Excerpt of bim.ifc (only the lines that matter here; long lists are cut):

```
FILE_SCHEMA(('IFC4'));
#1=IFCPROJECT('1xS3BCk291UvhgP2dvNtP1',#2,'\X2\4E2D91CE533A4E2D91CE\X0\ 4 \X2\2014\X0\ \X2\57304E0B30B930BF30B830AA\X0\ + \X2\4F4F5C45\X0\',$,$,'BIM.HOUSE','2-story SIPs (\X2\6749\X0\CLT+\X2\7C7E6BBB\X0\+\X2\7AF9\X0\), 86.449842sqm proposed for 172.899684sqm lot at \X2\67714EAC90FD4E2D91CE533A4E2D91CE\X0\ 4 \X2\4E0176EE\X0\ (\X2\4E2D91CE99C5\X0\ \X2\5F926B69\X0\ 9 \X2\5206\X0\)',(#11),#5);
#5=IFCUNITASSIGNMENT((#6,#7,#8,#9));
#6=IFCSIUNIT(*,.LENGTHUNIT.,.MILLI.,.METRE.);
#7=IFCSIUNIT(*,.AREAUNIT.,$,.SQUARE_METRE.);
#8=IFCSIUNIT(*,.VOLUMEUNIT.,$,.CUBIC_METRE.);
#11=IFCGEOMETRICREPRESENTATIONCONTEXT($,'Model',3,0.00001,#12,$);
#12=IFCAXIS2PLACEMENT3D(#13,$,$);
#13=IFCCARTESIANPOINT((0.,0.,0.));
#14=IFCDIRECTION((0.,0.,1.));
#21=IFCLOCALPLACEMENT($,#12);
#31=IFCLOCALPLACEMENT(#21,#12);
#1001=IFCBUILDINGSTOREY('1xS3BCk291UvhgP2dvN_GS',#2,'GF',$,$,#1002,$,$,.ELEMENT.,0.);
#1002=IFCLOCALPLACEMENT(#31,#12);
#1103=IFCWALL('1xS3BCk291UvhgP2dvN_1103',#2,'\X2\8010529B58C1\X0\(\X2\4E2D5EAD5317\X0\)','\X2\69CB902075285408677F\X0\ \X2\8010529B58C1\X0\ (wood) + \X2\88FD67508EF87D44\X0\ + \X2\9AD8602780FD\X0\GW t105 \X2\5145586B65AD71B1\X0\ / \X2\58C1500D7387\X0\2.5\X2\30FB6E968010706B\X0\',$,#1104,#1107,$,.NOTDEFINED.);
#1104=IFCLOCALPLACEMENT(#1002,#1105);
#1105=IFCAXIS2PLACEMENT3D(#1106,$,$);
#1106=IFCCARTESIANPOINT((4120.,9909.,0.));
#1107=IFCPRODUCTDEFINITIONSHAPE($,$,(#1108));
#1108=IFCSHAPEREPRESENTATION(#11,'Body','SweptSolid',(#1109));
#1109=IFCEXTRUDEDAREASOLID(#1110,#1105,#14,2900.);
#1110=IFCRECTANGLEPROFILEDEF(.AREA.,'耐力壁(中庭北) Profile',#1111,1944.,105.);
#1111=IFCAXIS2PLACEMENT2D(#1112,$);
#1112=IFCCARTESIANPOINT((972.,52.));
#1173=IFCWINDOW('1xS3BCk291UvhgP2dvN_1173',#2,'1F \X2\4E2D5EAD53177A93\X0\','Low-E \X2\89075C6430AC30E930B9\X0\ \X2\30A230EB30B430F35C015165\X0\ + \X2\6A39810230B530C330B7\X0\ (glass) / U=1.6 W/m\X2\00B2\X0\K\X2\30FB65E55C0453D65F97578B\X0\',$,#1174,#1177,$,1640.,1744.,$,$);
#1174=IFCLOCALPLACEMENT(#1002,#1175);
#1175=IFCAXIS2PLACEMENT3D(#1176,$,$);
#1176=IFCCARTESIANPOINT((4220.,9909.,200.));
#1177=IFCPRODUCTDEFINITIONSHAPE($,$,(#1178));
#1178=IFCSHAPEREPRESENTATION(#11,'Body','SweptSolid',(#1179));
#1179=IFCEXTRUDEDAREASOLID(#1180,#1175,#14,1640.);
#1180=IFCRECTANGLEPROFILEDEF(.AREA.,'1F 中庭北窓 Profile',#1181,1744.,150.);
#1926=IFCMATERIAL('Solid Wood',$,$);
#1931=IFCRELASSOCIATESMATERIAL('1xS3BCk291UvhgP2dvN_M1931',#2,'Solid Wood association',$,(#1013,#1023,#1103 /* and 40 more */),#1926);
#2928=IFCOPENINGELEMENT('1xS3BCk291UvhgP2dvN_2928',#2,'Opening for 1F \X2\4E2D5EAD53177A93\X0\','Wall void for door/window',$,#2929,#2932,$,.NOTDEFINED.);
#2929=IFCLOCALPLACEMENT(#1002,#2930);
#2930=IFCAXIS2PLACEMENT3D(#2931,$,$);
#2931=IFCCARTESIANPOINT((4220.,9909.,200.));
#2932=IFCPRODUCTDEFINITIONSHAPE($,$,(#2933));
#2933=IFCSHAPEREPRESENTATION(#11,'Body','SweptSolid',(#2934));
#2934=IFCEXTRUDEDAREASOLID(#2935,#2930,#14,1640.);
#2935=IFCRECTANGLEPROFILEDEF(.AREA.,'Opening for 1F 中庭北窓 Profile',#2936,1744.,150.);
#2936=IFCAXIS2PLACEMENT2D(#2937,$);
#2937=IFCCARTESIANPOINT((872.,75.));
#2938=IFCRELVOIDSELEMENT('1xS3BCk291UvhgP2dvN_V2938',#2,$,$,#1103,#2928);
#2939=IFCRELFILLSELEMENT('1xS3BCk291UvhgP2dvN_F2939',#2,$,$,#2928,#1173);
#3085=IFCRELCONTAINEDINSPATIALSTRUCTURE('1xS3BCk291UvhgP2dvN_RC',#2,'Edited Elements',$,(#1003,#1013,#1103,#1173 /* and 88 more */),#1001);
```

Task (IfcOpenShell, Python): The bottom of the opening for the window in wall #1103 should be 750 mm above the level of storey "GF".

```python
import numpy as np
import ifcopenshell
import ifcopenshell.api.geometry
import ifcopenshell.geom
import ifcopenshell.util.element
import ifcopenshell.util.placement
import ifcopenshell.util.shape
import ifcopenshell.util.unit

model = ifcopenshell.open("bim.ifc")
unit_scale = ifcopenshell.util.unit.calculate_unit_scale(model)

window = model.by_id(1173)
opening = window.FillsVoids[0].RelatingOpeningElement
storey = ifcopenshell.util.element.get_container(window, ifc_class="IfcBuildingStorey")
level = ifcopenshell.util.placement.get_local_placement(storey.ObjectPlacement)[2, 3]

# The opening's origin need not be at the sill, so measure its lowest point.
shape = ifcopenshell.geom.create_shape(ifcopenshell.geom.settings(), opening)
bottom = ifcopenshell.util.shape.get_shape_bottom_elevation(shape, shape.geometry) / unit_scale
dz = level + 750.0 - bottom

shift = np.array([0.0, 0.0, dz])
# The window is not placed relative to its opening, so move both.
for product in (opening, window):
    matrix = ifcopenshell.util.placement.get_local_placement(product.ObjectPlacement)
    matrix[:3, 3] += shift
    ifcopenshell.api.geometry.edit_object_placement(model, product=product, matrix=matrix, is_si=False)

print(f"moved by {dz * unit_scale:+.3f} m")

model.write("bim_rev.ifc")
```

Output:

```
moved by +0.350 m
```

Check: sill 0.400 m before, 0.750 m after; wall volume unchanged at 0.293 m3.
